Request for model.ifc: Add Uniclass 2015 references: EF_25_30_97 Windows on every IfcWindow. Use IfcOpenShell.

First a look at what the model holds.

```python
import ifcopenshell

model = ifcopenshell.open("model.ifc")
print(model.schema)
print("classifications:", [c.Name for c in model.by_type("IfcClassification")])
for ifc_class in ("IfcDoor", "IfcRoof", "IfcStair", "IfcWall", "IfcWindow"):
    print(ifc_class, len(model.by_type(ifc_class)))
```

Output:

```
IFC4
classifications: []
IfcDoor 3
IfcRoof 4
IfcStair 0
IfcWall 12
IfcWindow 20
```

```python
import ifcopenshell
import ifcopenshell.api.classification

model = ifcopenshell.open("model.ifc")

system = ifcopenshell.api.classification.add_classification(model, classification="Uniclass 2015")

codes = {
    "IfcWindow": ("EF_25_30_97", "Windows"),
}
for ifc_class, (code, name) in codes.items():
    products = model.by_type(ifc_class)
    ifcopenshell.api.classification.add_reference(
        model, products=products, classification=system, identification=code, name=name
    )
    print(code, len(products))

model.write("model_updated.ifc")
```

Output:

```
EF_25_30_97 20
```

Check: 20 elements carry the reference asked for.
